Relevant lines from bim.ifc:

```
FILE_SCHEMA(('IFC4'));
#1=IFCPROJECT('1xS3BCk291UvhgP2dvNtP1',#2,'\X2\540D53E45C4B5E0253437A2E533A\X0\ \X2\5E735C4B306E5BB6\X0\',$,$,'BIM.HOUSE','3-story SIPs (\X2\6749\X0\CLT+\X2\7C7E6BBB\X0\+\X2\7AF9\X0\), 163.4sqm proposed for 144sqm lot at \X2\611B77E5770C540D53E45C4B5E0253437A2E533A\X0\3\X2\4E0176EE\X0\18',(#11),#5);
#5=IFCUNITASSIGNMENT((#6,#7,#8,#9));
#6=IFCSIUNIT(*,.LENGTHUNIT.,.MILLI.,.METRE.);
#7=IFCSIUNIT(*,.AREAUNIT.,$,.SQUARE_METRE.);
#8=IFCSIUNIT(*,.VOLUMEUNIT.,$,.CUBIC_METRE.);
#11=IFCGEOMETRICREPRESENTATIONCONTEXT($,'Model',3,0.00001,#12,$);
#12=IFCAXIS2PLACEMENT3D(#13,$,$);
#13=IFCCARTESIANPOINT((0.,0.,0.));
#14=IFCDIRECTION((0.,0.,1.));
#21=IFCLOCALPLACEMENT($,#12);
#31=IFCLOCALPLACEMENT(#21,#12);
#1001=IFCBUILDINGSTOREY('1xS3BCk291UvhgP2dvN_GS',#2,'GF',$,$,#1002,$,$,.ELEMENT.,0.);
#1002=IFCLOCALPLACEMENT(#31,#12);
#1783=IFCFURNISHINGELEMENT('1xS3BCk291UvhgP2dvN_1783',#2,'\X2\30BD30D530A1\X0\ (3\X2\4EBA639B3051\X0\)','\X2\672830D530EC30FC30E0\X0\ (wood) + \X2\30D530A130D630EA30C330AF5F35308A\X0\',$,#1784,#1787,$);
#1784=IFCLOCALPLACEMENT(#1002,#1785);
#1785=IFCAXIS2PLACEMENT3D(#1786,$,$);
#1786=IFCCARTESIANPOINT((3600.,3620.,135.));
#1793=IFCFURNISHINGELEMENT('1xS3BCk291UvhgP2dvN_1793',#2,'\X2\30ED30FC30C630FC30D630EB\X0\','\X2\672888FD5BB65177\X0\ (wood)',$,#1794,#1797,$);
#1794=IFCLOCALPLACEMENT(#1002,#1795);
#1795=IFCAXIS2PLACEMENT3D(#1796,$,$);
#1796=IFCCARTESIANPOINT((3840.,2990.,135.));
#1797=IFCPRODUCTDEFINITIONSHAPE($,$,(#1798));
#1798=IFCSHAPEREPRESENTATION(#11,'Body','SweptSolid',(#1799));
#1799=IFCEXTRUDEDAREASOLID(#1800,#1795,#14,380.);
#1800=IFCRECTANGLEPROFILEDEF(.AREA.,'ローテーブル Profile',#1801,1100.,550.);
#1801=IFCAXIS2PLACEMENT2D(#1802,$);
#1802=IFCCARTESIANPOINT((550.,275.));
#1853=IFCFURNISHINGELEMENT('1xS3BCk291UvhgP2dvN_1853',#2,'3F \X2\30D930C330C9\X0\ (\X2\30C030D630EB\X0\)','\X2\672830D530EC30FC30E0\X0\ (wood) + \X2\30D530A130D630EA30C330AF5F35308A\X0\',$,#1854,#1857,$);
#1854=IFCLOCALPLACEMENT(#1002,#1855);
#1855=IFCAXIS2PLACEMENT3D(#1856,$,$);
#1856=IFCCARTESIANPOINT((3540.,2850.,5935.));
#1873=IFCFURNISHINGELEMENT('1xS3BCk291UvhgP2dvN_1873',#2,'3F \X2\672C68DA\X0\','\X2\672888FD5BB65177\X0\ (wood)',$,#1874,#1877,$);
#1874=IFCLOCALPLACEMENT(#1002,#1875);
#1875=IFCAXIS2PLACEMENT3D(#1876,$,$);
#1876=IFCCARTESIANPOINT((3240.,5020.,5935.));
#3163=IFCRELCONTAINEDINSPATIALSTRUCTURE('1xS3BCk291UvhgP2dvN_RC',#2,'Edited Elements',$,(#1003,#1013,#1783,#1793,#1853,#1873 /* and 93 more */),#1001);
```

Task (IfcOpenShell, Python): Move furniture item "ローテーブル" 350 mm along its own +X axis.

```python
import ifcopenshell
import ifcopenshell.api.geometry
import ifcopenshell.util.placement
import ifcopenshell.util.unit

model = ifcopenshell.open("bim.ifc")
unit_scale = ifcopenshell.util.unit.calculate_unit_scale(model)

item = model.by_id(1793)
matrix = ifcopenshell.util.placement.get_local_placement(item.ObjectPlacement)
matrix[:3, 3] += matrix[:3, 0] * 0.35 / unit_scale
ifcopenshell.api.geometry.edit_object_placement(model, product=item, matrix=matrix, is_si=False)

print(ifcopenshell.util.placement.get_local_placement(item.ObjectPlacement).round(3) + 0.0)

model.write("bim_rev.ifc")
```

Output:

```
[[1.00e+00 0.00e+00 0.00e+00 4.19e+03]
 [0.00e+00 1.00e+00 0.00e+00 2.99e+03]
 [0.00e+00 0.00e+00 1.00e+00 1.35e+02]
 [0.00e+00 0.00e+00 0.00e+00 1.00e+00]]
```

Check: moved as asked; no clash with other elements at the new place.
